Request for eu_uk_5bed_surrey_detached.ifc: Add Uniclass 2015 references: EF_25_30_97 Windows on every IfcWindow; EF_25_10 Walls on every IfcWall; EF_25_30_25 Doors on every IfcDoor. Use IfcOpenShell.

First a look at what the model holds.

```python
import ifcopenshell

model = ifcopenshell.open("eu_uk_5bed_surrey_detached.ifc")
print(model.schema)
print("classifications:", [c.Name for c in model.by_type("IfcClassification")])
for ifc_class in ("IfcDoor", "IfcRoof", "IfcStair", "IfcWall", "IfcWindow"):
    print(ifc_class, len(model.by_type(ifc_class)))
```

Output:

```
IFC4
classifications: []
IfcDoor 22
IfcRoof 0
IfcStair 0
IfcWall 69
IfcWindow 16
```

```python
import ifcopenshell
import ifcopenshell.api.classification

model = ifcopenshell.open("eu_uk_5bed_surrey_detached.ifc")

system = ifcopenshell.api.classification.add_classification(model, classification="Uniclass 2015")

codes = {
    "IfcWindow": ("EF_25_30_97", "Windows"),
    "IfcWall": ("EF_25_10", "Walls"),
    "IfcDoor": ("EF_25_30_25", "Doors"),
}
for ifc_class, (code, name) in codes.items():
    products = model.by_type(ifc_class)
    ifcopenshell.api.classification.add_reference(
        model, products=products, classification=system, identification=code, name=name
    )
    print(code, len(products))

model.write("eu_uk_5bed_surrey_detached_edited.ifc")
```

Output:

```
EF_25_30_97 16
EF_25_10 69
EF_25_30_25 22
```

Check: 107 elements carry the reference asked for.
